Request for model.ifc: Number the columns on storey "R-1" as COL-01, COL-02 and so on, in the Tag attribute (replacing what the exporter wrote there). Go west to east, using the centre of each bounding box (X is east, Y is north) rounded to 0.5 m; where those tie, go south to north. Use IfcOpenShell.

First a look at what the model holds.

```python
import ifcopenshell
import ifcopenshell.util.element
import ifcopenshell.util.placement

model = ifcopenshell.open("model.ifc")
print(model.schema)
storey = next(s for s in model.by_type("IfcBuildingStorey") if s.Name == "R-1")
columns = [e for e in ifcopenshell.util.element.get_decomposition(storey) if e.is_a("IfcColumn")]
for e in sorted(columns, key=lambda e: e.id()):
    origin = ifcopenshell.util.placement.get_local_placement(e.ObjectPlacement)[:3, 3]
    print(e.id(), e.Tag, e.Name, origin.round(2) + 0.0, sep=" | ")
```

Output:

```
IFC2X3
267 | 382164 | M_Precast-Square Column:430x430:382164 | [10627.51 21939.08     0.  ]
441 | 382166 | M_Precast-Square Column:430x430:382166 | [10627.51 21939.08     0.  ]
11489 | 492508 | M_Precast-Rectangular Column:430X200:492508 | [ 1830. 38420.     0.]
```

```python
import ifcopenshell
import ifcopenshell.geom
import ifcopenshell.util.element
import ifcopenshell.util.shape

model = ifcopenshell.open("model.ifc")
settings = ifcopenshell.geom.settings()
settings.set("use-world-coords", True)


def centre(element):
    shape = ifcopenshell.geom.create_shape(settings, element)
    return ifcopenshell.util.shape.get_bbox_centroid(shape.geometry)


storey = next(s for s in model.by_type("IfcBuildingStorey") if s.Name == "R-1")
columns = [e for e in ifcopenshell.util.element.get_decomposition(storey) if e.is_a("IfcColumn")]

# Insertion points can sit at a corner or the storey origin, so sort by the geometry (in metres).
centres = {e: centre(e) for e in columns}
columns.sort(key=lambda e: (round(centres[e][0] / 0.5), centres[e][1]))

for i, e in enumerate(columns, start=1):
    number = f"COL-{i:02d}"
    e.Tag = number
    print(e.id(), number)

model.write("model_edited.ifc")
```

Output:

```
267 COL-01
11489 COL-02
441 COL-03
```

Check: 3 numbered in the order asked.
